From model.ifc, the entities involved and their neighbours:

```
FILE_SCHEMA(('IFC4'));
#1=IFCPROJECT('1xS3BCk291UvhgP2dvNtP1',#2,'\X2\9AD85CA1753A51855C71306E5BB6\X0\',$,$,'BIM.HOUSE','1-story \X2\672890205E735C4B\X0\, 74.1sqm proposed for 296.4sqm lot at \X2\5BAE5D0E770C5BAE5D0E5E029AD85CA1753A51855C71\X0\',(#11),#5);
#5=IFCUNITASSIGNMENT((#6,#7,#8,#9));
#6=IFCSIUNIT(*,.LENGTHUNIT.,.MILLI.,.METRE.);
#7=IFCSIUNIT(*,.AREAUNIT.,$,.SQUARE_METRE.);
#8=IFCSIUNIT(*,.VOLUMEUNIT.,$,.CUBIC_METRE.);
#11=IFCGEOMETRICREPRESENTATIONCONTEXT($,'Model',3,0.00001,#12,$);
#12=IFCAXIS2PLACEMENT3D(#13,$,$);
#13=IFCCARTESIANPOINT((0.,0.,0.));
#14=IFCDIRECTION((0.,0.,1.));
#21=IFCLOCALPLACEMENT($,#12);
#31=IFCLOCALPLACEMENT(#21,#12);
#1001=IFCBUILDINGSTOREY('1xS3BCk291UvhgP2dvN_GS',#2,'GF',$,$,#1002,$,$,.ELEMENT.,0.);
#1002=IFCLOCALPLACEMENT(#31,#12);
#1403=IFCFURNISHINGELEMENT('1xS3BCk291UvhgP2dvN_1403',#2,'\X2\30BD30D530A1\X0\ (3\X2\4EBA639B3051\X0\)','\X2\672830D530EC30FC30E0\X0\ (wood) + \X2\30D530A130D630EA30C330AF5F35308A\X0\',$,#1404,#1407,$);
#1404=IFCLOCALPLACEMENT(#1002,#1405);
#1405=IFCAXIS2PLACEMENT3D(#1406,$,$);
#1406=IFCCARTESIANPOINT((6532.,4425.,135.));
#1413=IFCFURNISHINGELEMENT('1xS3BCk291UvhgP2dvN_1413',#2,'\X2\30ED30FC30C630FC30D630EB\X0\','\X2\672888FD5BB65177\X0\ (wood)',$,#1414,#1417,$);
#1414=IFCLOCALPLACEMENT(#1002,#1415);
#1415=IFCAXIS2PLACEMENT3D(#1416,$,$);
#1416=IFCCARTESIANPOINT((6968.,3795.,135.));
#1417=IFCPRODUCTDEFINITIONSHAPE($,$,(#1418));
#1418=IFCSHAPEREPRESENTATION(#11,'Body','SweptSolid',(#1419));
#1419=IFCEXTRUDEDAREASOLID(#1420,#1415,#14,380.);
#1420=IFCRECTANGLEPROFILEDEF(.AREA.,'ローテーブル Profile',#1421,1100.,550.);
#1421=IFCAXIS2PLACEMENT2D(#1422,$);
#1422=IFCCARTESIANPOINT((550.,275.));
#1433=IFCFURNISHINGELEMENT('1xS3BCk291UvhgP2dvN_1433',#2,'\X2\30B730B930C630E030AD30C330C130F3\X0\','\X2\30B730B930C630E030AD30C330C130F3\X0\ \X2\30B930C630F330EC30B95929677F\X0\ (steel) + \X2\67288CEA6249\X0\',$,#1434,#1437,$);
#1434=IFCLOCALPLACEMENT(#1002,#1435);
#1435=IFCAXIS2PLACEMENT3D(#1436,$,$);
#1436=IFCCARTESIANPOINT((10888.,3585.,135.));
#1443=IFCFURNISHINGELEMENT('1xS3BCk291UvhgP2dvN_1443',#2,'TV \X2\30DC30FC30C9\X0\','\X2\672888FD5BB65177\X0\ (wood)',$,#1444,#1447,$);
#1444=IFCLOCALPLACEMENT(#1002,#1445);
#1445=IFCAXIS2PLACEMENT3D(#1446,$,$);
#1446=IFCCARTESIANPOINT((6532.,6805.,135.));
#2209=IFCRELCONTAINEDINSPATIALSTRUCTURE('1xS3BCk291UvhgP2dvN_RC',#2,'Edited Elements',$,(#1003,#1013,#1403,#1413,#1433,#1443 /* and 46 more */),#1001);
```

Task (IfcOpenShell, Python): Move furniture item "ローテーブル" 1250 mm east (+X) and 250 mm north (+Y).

```python
import ifcopenshell
import ifcopenshell.api.geometry
import ifcopenshell.util.placement

model = ifcopenshell.open("model.ifc")

item = model.by_id(1413)
matrix = ifcopenshell.util.placement.get_local_placement(item.ObjectPlacement)
matrix[0, 3] += 1250.0
matrix[1, 3] += 250.0
ifcopenshell.api.geometry.edit_object_placement(model, product=item, matrix=matrix, is_si=False)

print(ifcopenshell.util.placement.get_local_placement(item.ObjectPlacement).round(3) + 0.0)

model.write("model_updated.ifc")
```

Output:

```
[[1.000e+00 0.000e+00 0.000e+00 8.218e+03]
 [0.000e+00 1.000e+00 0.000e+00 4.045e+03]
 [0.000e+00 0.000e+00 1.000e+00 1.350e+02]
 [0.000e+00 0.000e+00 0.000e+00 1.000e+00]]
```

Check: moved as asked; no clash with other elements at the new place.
